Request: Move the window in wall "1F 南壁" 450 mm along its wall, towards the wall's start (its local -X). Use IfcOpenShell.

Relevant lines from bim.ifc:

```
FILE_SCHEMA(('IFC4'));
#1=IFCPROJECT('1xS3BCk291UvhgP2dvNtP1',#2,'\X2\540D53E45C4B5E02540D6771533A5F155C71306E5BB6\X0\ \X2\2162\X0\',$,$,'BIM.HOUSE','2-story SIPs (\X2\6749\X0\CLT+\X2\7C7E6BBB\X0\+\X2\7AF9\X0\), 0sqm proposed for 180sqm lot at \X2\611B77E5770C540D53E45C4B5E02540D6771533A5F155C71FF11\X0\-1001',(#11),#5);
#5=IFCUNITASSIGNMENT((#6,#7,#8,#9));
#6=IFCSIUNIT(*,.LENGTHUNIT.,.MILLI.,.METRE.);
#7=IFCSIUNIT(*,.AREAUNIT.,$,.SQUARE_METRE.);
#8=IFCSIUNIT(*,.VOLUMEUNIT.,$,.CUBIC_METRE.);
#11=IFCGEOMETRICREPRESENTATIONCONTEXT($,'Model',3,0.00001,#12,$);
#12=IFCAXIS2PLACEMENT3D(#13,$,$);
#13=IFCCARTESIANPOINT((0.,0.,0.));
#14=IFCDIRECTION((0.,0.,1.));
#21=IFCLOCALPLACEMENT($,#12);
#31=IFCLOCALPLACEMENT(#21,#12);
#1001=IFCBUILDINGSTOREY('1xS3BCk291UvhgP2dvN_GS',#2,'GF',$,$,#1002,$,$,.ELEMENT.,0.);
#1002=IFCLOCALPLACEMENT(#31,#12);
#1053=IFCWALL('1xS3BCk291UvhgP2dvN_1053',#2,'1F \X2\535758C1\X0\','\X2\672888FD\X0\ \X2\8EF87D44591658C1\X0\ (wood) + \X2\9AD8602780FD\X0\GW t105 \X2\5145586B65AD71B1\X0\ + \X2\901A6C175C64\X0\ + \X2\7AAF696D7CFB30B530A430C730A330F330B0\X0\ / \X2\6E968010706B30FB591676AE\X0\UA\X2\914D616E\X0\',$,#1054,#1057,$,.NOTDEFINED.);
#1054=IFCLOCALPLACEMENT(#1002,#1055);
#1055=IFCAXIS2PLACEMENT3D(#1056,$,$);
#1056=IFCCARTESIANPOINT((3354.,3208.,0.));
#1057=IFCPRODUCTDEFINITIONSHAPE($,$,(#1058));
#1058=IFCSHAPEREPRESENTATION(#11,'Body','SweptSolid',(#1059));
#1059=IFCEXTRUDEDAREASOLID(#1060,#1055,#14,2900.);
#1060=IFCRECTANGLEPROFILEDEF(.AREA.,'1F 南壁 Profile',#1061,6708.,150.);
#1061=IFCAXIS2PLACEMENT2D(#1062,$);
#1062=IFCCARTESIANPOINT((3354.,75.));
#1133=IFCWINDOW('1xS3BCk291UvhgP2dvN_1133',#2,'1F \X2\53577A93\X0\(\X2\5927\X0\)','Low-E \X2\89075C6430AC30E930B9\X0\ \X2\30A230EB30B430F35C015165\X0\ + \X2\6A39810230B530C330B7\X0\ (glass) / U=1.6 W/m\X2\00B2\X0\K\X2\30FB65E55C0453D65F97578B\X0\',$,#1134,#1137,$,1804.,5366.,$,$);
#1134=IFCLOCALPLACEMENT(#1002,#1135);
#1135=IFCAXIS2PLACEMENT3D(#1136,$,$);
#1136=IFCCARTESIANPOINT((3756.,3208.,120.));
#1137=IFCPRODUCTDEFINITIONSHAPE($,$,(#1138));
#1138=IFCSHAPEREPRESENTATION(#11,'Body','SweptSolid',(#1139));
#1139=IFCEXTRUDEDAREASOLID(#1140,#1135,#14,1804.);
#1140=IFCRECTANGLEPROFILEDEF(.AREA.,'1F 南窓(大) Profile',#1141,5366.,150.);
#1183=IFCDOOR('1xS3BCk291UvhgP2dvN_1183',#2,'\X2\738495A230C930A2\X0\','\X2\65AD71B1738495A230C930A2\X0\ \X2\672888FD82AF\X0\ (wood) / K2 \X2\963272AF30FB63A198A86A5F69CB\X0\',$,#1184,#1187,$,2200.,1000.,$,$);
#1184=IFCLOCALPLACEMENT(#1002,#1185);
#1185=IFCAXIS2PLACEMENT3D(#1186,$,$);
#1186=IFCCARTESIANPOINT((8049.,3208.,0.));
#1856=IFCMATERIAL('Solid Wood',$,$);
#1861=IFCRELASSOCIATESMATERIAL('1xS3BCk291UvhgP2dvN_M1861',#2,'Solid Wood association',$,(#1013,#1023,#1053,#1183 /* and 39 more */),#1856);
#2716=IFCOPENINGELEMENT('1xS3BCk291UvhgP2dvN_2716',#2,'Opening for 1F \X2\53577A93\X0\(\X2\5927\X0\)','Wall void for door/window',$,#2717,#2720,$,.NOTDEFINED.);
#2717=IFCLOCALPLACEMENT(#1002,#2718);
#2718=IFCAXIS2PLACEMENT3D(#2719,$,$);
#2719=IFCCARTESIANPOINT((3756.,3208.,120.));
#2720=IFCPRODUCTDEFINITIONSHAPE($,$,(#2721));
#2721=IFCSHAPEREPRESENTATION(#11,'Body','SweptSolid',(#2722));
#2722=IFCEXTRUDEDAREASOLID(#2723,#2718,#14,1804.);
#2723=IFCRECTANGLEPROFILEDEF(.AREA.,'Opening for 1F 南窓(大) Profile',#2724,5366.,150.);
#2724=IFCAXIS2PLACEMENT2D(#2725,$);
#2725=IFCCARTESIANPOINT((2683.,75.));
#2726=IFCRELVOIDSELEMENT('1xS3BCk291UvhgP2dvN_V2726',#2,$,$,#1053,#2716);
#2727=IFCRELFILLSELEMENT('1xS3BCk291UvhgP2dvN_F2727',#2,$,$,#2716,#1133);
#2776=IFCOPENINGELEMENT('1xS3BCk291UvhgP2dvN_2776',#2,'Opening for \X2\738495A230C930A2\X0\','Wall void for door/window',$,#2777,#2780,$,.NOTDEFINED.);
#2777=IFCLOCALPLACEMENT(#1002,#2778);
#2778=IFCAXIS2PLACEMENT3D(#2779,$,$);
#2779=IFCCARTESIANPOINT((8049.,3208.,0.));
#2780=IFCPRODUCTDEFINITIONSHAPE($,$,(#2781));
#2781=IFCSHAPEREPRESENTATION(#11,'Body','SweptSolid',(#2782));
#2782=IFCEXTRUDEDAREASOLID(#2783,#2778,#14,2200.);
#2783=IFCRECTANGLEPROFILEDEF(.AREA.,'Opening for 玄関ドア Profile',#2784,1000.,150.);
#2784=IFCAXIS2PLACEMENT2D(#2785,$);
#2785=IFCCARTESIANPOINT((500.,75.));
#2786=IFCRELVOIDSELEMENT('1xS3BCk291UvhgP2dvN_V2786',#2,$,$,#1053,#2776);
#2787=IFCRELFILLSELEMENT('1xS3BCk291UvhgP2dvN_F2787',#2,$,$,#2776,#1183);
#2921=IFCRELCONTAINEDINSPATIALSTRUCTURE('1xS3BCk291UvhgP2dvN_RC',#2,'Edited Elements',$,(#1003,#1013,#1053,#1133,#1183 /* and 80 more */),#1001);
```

```python
import ifcopenshell
import ifcopenshell.api.geometry
import ifcopenshell.util.placement
import ifcopenshell.util.unit

model = ifcopenshell.open("bim.ifc")
unit_scale = ifcopenshell.util.unit.calculate_unit_scale(model)

window = model.by_guid("1xS3BCk291UvhgP2dvN_1133")
opening = window.FillsVoids[0].RelatingOpeningElement
wall = opening.VoidsElements[0].RelatingBuildingElement

wall_matrix = ifcopenshell.util.placement.get_local_placement(wall.ObjectPlacement)
shift = wall_matrix[:3, 0] * -0.45 / unit_scale
before = ifcopenshell.util.placement.get_local_placement(window.ObjectPlacement)[:3, 3].copy()

# The window is not placed relative to its opening, so move both.
for product in (opening, window):
    matrix = ifcopenshell.util.placement.get_local_placement(product.ObjectPlacement)
    matrix[:3, 3] += shift
    ifcopenshell.api.geometry.edit_object_placement(model, product=product, matrix=matrix, is_si=False)

after = ifcopenshell.util.placement.get_local_placement(window.ObjectPlacement)[:3, 3]
print("window moved by", (after - before).round(3) + 0.0)

model.write("bim_v2.ifc")
```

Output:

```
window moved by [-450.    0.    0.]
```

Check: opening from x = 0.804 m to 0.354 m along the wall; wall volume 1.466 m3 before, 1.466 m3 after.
